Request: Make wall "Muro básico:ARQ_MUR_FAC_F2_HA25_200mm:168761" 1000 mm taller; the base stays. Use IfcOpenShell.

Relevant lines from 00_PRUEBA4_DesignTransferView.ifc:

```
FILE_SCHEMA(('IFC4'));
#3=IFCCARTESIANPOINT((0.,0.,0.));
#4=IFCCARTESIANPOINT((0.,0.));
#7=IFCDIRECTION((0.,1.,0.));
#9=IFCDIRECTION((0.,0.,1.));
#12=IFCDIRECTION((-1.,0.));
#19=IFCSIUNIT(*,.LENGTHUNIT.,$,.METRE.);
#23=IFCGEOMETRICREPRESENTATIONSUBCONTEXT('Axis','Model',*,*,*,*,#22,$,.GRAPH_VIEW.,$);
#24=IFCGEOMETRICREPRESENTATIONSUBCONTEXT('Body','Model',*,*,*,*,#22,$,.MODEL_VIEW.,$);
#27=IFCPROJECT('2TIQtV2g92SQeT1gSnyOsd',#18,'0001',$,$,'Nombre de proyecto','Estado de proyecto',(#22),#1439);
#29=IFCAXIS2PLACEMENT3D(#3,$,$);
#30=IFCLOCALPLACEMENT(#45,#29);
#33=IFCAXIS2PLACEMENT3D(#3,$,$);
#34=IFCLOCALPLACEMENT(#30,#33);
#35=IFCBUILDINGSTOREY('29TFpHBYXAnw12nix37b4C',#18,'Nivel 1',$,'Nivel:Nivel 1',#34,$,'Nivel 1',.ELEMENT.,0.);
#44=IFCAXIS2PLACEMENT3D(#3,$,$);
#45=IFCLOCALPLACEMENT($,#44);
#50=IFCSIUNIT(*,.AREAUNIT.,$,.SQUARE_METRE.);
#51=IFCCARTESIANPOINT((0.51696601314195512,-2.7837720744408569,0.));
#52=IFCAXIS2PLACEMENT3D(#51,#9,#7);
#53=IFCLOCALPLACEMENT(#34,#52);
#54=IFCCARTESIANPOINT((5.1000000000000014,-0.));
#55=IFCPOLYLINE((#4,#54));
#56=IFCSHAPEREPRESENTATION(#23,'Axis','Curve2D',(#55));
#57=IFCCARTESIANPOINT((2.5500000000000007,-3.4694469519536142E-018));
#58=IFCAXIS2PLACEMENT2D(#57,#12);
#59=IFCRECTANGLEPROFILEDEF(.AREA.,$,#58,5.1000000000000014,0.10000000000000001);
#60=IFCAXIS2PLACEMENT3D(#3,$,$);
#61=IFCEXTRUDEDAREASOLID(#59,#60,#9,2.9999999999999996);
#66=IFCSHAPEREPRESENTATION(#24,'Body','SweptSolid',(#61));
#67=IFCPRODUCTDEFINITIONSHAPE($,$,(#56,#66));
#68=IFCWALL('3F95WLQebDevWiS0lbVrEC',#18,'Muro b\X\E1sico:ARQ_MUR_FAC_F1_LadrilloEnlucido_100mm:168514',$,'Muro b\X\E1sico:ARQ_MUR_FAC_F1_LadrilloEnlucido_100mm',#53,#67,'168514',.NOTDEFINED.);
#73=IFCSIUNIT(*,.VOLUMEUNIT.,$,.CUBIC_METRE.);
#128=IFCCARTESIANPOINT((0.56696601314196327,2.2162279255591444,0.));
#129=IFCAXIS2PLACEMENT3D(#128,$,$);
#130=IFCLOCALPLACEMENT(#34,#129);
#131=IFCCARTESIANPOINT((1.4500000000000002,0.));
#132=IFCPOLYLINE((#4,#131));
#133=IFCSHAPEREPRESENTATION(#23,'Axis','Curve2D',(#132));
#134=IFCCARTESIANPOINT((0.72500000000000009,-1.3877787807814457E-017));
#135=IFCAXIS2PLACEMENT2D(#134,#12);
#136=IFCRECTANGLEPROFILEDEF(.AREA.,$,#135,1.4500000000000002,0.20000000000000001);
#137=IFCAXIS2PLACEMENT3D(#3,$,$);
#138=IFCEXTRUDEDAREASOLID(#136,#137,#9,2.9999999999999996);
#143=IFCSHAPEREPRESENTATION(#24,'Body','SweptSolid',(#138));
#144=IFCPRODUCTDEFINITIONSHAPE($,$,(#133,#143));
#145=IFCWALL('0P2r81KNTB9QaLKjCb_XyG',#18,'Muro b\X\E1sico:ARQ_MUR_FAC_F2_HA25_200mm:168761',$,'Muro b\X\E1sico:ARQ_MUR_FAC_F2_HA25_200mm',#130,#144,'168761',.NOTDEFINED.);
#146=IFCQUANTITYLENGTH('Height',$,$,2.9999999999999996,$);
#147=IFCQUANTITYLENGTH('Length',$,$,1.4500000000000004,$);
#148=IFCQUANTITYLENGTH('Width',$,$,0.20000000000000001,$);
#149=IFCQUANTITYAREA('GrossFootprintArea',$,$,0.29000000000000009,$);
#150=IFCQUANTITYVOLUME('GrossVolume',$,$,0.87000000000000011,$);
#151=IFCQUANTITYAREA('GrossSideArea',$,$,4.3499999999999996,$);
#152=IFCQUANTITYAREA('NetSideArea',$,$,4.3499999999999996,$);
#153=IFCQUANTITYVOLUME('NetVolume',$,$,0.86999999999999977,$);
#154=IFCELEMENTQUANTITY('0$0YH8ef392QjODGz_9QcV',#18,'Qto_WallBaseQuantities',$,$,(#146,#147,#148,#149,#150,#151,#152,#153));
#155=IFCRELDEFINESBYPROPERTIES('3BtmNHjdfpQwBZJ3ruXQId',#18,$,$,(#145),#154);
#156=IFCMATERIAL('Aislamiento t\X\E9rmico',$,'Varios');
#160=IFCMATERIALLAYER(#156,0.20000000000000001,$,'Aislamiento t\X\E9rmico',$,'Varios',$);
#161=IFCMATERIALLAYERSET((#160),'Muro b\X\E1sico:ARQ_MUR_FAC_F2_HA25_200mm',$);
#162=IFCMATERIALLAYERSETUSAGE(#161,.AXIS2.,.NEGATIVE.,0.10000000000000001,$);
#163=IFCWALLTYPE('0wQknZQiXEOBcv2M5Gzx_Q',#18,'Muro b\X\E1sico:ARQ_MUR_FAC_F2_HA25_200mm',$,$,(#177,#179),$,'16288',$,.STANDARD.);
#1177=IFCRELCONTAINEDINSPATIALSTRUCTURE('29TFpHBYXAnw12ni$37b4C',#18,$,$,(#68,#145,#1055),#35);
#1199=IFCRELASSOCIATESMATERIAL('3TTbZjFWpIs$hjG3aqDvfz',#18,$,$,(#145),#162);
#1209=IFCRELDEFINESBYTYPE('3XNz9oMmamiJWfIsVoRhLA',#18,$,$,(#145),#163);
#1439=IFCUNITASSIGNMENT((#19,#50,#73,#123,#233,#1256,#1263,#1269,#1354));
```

```python
import ifcopenshell
import ifcopenshell.api.pset
import ifcopenshell.geom
import ifcopenshell.util.element
import ifcopenshell.util.representation
import ifcopenshell.util.shape
import ifcopenshell.util.unit

model = ifcopenshell.open("00_PRUEBA4_DesignTransferView.ifc")
unit_scale = ifcopenshell.util.unit.calculate_unit_scale(model)
area_scale = ifcopenshell.util.unit.calculate_unit_scale(model, "AREAUNIT")
volume_scale = ifcopenshell.util.unit.calculate_unit_scale(model, "VOLUMEUNIT")
settings = ifcopenshell.geom.settings()


def volume(element):
    """Net volume in cubic metres, openings subtracted."""
    shape = ifcopenshell.geom.create_shape(settings, element)
    return ifcopenshell.util.shape.get_volume(shape.geometry)


wall = model.by_guid("0P2r81KNTB9QaLKjCb_XyG")
before = volume(wall)

body = ifcopenshell.util.representation.get_representation(wall, "Model", "Body")
solid = body.Items[0]
old_height = solid.Depth
solid.Depth += 1.0
after = volume(wall)
thickness = 0.2  # wall thickness in metres

# Update the stored height, areas and volumes.
qto = model.by_id(ifcopenshell.util.element.get_pset(wall, "Qto_WallBaseQuantities", should_inherit=False)["id"])
ifcopenshell.api.pset.edit_qto(model, qto=qto, properties={
    "Height": solid.Depth,
    "GrossVolume": ifcopenshell.util.element.get_pset(wall, "Qto_WallBaseQuantities", "GrossVolume") * solid.Depth / old_height,
    "GrossSideArea": ifcopenshell.util.element.get_pset(wall, "Qto_WallBaseQuantities", "GrossSideArea") * solid.Depth / old_height,
    "NetSideArea": after / thickness / area_scale,
    "NetVolume": after / volume_scale,
})

print(f"height {old_height:g} -> {solid.Depth:g}, volume {before:.3f} -> {after:.3f} m3")

model.write("00_PRUEBA4_DesignTransferView_rev.ifc")
```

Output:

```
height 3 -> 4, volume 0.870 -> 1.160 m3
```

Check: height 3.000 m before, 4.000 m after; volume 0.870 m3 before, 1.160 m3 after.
